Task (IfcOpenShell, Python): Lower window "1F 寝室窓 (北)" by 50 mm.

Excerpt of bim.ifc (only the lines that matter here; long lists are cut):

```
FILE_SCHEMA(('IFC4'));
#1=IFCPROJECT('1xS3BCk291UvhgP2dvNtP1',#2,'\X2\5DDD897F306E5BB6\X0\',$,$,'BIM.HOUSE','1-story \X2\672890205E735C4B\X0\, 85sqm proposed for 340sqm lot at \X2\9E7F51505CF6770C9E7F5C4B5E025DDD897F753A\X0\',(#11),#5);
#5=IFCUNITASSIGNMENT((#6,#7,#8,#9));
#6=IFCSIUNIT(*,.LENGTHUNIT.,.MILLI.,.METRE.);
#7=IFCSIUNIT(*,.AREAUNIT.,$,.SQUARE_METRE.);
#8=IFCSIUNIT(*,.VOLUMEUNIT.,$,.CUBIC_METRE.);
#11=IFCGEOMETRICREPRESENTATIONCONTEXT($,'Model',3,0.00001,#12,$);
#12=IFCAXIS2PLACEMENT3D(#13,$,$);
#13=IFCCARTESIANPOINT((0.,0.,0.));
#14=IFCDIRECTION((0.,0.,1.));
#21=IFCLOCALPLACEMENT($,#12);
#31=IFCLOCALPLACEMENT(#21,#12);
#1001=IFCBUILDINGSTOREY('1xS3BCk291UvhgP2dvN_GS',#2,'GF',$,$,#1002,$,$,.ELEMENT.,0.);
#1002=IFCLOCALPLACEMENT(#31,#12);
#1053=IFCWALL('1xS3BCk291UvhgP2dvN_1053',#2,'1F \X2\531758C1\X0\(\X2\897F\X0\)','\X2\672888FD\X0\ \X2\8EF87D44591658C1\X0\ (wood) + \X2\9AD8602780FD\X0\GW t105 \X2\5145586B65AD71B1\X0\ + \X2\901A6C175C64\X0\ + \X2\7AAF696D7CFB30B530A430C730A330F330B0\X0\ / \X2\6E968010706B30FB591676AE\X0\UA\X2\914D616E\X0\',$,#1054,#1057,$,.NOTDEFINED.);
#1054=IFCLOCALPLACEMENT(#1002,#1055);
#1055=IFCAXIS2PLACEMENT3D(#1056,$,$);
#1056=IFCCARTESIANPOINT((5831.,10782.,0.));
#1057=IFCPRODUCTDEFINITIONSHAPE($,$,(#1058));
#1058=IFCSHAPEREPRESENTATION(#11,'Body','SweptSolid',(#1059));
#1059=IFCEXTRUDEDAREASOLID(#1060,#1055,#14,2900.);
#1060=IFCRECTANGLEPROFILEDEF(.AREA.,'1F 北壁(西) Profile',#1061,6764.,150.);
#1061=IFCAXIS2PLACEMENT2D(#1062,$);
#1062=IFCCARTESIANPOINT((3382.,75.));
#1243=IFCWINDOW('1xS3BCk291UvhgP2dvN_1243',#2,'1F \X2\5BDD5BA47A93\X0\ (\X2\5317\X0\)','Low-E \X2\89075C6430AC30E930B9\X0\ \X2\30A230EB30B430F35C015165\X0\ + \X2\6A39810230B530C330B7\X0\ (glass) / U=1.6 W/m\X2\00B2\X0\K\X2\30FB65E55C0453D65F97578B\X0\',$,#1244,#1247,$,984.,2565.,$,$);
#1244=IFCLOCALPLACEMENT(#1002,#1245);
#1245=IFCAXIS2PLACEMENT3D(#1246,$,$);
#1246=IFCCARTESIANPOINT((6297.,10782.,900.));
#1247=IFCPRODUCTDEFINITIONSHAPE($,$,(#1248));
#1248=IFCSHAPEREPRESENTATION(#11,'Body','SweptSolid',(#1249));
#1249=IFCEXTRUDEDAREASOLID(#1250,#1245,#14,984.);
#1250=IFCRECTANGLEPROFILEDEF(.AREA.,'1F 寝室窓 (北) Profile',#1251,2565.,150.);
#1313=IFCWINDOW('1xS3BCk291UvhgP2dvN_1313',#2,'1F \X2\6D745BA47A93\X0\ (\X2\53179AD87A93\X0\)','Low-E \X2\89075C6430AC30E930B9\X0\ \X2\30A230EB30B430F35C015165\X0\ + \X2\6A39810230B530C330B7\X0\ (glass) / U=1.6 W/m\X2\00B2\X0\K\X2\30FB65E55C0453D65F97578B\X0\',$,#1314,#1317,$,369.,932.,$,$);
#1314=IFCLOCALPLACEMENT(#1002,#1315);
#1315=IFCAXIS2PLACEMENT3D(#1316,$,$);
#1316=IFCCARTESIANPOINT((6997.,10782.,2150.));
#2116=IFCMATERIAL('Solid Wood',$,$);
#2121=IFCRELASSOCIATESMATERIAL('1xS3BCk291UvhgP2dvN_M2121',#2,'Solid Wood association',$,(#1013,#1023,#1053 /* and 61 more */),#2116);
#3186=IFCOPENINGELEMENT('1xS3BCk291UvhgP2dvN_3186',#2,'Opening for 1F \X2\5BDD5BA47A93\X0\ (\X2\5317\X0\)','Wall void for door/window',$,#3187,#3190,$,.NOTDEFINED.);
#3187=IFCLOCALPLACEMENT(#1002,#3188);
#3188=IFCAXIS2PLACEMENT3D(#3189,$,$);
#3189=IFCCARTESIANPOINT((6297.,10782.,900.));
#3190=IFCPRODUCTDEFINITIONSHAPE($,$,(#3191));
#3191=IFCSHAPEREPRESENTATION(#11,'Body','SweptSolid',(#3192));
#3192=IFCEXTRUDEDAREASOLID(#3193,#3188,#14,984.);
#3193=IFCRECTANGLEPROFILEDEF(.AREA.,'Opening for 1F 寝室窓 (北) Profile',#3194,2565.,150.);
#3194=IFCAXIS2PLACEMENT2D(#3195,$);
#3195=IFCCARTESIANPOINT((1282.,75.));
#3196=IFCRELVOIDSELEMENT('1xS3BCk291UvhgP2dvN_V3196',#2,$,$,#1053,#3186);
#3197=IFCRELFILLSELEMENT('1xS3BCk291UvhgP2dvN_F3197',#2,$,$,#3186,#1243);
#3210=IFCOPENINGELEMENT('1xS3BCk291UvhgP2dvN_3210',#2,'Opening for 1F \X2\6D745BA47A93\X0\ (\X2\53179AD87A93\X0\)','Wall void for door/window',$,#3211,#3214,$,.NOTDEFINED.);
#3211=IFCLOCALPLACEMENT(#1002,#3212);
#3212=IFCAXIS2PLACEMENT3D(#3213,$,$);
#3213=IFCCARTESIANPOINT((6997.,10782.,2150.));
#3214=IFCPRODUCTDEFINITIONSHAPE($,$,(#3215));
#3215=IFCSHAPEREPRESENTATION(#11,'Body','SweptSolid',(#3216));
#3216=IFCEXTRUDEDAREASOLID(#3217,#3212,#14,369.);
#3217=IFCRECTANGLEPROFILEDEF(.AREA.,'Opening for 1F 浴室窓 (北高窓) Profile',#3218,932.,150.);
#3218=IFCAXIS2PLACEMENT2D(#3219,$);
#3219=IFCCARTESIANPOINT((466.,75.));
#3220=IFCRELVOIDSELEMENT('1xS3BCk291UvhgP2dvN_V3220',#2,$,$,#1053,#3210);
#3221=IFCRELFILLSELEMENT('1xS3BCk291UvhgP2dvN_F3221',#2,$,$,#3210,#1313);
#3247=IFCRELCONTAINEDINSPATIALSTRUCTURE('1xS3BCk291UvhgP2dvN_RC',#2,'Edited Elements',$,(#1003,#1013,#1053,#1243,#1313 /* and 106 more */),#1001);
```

```python
import numpy as np
import ifcopenshell
import ifcopenshell.api.geometry
import ifcopenshell.util.placement
import ifcopenshell.util.unit

model = ifcopenshell.open("bim.ifc")
unit_scale = ifcopenshell.util.unit.calculate_unit_scale(model)

window = model.by_id(1243)
opening = window.FillsVoids[0].RelatingOpeningElement
dz = -0.05 / unit_scale

shift = np.array([0.0, 0.0, dz])
# The window is not placed relative to its opening, so move both.
for product in (opening, window):
    matrix = ifcopenshell.util.placement.get_local_placement(product.ObjectPlacement)
    matrix[:3, 3] += shift
    ifcopenshell.api.geometry.edit_object_placement(model, product=product, matrix=matrix, is_si=False)

print(f"moved by {dz * unit_scale:+.3f} m")

model.write("bim-out.ifc")
```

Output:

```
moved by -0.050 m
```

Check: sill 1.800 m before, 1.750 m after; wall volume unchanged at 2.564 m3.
